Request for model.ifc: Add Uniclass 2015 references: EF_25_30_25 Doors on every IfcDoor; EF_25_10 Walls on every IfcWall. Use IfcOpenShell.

First a look at what the model holds.

```python
import ifcopenshell

model = ifcopenshell.open("model.ifc")
print(model.schema)
print("classifications:", [c.Name for c in model.by_type("IfcClassification")])
for ifc_class in ("IfcDoor", "IfcRoof", "IfcStair", "IfcWall", "IfcWindow"):
    print(ifc_class, len(model.by_type(ifc_class)))
```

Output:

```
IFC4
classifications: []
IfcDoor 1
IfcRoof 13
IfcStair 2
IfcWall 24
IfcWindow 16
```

```python
import ifcopenshell
import ifcopenshell.api.classification

model = ifcopenshell.open("model.ifc")

system = ifcopenshell.api.classification.add_classification(model, classification="Uniclass 2015")

codes = {
    "IfcDoor": ("EF_25_30_25", "Doors"),
    "IfcWall": ("EF_25_10", "Walls"),
}
for ifc_class, (code, name) in codes.items():
    products = model.by_type(ifc_class)
    ifcopenshell.api.classification.add_reference(
        model, products=products, classification=system, identification=code, name=name
    )
    print(code, len(products))

model.write("model_edited.ifc")
```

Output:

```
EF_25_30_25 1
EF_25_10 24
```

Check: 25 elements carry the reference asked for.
